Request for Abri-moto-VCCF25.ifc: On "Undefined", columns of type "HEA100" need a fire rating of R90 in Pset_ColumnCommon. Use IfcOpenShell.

First a look at what the model holds.

```python
import ifcopenshell
import ifcopenshell.util.element

model = ifcopenshell.open("Abri-moto-VCCF25.ifc")
print(model.schema)
storey = next(s for s in model.by_type("IfcBuildingStorey") if s.Name == "Undefined")
columns = [e for e in ifcopenshell.util.element.get_decomposition(storey) if e.is_a("IfcColumn")]
seen = {}
for e in columns:
    element_type = ifcopenshell.util.element.get_type(e)
    key = (element_type.Name if element_type != e and element_type else None, ifcopenshell.util.element.get_pset(e, "Pset_ColumnCommon", "FireRating"))
    seen[key] = seen.get(key, 0) + 1
for (name, value), count in sorted(seen.items(), key=str):
    print(count, "x", name, "|", value)
```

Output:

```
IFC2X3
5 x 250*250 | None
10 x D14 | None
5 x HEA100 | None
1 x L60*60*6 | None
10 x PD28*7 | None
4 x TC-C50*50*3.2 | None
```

```python
import ifcopenshell
import ifcopenshell.api.pset
import ifcopenshell.util.element

model = ifcopenshell.open("Abri-moto-VCCF25.ifc")

storey = next(s for s in model.by_type("IfcBuildingStorey") if s.Name == "Undefined")
columns = [e for e in ifcopenshell.util.element.get_decomposition(storey) if e.is_a("IfcColumn")]

count = 0
for e in columns:
    element_type = ifcopenshell.util.element.get_type(e)
    if element_type in (None, e) or element_type.Name != "HEA100":
        continue
    # add_pset returns the element's existing set when there is one.
    pset = ifcopenshell.api.pset.add_pset(model, product=e, name="Pset_ColumnCommon")
    ifcopenshell.api.pset.edit_pset(model, pset=pset, properties={"FireRating": "R90"})
    count += 1

print(count, "columns updated")

model.write("Abri-moto-VCCF25_v2.ifc")
```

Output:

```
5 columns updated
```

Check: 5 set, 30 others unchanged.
